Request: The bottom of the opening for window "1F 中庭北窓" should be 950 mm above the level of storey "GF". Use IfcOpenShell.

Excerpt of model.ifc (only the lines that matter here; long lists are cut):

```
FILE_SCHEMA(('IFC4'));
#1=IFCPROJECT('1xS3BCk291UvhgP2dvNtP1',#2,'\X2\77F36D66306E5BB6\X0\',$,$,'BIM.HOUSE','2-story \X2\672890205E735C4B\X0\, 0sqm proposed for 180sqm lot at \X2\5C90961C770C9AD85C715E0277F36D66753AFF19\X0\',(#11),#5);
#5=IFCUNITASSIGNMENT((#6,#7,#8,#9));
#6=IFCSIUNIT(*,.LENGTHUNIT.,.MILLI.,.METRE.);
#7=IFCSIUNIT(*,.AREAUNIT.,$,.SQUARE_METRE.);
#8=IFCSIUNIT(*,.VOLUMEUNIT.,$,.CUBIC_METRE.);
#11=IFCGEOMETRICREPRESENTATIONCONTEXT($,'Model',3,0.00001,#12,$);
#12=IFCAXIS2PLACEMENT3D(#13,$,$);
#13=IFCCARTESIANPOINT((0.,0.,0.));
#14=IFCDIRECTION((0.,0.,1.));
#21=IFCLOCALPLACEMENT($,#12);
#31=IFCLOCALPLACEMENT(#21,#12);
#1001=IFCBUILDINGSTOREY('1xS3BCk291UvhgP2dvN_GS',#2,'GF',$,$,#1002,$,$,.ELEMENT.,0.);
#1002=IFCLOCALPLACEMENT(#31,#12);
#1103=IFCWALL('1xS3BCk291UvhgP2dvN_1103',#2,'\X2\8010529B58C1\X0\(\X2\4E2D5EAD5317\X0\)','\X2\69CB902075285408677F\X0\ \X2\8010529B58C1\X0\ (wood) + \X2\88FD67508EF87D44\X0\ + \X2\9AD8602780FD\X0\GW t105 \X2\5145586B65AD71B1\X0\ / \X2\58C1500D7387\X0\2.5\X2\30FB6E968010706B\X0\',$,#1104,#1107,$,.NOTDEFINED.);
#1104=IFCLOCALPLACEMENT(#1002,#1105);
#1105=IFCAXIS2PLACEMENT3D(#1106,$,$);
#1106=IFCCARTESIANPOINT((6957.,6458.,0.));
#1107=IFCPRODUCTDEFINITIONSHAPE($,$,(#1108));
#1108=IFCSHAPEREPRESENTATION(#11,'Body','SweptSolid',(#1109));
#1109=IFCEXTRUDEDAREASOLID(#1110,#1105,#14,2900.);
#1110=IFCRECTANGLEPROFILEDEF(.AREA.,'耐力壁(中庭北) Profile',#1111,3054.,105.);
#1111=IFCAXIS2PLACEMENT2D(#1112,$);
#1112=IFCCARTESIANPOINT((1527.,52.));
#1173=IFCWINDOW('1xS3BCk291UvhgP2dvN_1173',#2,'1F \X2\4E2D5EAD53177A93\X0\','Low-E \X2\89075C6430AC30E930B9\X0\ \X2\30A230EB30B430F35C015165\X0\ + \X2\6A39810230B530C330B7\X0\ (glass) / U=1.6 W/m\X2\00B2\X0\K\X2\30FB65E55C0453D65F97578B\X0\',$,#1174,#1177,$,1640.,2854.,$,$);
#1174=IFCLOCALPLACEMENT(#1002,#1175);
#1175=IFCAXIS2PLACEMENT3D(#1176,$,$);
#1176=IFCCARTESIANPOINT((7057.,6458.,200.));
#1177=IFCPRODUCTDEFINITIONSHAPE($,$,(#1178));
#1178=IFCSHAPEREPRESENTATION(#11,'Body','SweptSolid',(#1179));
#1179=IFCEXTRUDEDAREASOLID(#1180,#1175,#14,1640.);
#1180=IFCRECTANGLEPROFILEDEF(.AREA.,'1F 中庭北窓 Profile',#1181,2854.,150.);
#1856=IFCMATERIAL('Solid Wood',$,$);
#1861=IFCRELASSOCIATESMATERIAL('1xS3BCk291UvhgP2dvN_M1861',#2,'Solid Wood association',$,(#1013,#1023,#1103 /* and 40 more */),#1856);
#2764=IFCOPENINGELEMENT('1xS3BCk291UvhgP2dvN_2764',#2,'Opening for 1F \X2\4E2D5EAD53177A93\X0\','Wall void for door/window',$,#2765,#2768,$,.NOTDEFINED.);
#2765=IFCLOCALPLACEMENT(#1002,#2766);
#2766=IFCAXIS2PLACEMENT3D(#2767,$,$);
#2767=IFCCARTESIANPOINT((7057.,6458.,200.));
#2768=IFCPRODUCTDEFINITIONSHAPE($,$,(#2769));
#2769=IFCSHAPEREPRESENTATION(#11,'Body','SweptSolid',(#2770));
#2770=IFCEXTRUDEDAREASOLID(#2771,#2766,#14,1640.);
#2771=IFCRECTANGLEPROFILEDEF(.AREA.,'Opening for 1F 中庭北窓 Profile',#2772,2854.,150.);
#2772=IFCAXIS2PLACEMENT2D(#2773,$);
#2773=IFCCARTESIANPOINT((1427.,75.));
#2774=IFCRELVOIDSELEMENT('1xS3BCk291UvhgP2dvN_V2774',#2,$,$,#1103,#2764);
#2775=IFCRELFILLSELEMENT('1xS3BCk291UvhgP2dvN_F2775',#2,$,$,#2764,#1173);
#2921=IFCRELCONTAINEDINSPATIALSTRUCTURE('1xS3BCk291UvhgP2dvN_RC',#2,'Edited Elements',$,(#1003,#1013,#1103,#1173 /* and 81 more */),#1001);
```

```python
import numpy as np
import ifcopenshell
import ifcopenshell.api.geometry
import ifcopenshell.geom
import ifcopenshell.util.element
import ifcopenshell.util.placement
import ifcopenshell.util.shape
import ifcopenshell.util.unit

model = ifcopenshell.open("model.ifc")
unit_scale = ifcopenshell.util.unit.calculate_unit_scale(model)

window = model.by_guid("1xS3BCk291UvhgP2dvN_1173")
opening = window.FillsVoids[0].RelatingOpeningElement
storey = ifcopenshell.util.element.get_container(window, ifc_class="IfcBuildingStorey")
level = ifcopenshell.util.placement.get_local_placement(storey.ObjectPlacement)[2, 3]

# The opening's origin need not be at the sill, so measure its lowest point.
shape = ifcopenshell.geom.create_shape(ifcopenshell.geom.settings(), opening)
bottom = ifcopenshell.util.shape.get_shape_bottom_elevation(shape, shape.geometry) / unit_scale
dz = level + 0.95 / unit_scale - bottom

shift = np.array([0.0, 0.0, dz])
# The window is not placed relative to its opening, so move both.
for product in (opening, window):
    matrix = ifcopenshell.util.placement.get_local_placement(product.ObjectPlacement)
    matrix[:3, 3] += shift
    ifcopenshell.api.geometry.edit_object_placement(model, product=product, matrix=matrix, is_si=False)

print(f"moved by {dz * unit_scale:+.3f} m")

model.write("model_edited.ifc")
```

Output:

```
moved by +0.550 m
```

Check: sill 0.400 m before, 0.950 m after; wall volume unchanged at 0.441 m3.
